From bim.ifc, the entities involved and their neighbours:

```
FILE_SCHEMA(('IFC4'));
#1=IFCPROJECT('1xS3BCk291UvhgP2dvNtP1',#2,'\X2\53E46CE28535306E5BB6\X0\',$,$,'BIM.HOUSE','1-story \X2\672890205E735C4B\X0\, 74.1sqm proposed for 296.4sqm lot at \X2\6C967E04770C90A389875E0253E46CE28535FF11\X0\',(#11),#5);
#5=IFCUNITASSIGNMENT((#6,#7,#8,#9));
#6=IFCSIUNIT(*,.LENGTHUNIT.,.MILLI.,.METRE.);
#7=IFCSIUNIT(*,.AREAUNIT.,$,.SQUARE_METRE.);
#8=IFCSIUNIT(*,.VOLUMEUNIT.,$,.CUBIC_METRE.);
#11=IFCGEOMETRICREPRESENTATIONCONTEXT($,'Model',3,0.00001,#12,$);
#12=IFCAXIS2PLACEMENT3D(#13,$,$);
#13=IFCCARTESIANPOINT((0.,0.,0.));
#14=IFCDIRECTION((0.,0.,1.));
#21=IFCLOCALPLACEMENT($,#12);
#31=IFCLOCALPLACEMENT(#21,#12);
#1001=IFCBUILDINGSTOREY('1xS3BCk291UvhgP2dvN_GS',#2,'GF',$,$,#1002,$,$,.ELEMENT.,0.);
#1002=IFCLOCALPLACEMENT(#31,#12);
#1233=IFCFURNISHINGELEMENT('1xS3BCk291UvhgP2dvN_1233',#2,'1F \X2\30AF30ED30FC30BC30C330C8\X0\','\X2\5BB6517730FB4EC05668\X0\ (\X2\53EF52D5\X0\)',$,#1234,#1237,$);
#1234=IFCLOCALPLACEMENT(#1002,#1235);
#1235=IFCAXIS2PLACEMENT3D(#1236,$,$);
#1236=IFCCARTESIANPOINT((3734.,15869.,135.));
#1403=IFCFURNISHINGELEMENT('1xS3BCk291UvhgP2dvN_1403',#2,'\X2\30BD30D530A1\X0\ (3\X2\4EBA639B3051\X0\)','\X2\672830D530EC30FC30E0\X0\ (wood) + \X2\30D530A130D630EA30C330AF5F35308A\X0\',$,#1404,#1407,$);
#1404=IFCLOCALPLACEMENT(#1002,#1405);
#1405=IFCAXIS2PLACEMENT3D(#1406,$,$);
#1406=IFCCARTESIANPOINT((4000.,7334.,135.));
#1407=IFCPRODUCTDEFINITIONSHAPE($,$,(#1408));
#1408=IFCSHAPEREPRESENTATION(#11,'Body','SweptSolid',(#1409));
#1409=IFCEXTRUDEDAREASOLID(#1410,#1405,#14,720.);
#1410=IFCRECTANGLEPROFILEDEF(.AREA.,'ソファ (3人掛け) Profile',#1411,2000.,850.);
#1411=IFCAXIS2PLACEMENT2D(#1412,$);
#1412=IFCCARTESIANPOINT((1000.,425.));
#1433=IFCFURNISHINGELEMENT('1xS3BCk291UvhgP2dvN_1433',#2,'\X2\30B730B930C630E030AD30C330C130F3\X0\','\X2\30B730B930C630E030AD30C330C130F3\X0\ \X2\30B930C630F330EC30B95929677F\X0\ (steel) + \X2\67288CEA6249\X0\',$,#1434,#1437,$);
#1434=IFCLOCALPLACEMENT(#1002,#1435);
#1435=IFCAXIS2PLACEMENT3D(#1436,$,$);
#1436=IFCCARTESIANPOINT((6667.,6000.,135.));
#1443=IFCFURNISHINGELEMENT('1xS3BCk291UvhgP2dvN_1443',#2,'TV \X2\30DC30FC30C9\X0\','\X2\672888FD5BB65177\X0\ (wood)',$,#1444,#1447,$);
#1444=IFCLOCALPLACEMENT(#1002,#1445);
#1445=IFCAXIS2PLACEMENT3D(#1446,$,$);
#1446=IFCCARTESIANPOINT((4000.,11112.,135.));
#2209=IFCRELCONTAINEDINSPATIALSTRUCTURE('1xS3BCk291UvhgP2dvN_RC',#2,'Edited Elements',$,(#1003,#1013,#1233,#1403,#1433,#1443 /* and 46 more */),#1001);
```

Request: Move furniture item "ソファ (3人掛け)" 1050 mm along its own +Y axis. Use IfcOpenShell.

```python
import ifcopenshell
import ifcopenshell.api.geometry
import ifcopenshell.util.placement
import ifcopenshell.util.unit

model = ifcopenshell.open("bim.ifc")
unit_scale = ifcopenshell.util.unit.calculate_unit_scale(model)

item = model.by_id(1403)
matrix = ifcopenshell.util.placement.get_local_placement(item.ObjectPlacement)
matrix[:3, 3] += matrix[:3, 1] * 1.05 / unit_scale
ifcopenshell.api.geometry.edit_object_placement(model, product=item, matrix=matrix, is_si=False)

print(ifcopenshell.util.placement.get_local_placement(item.ObjectPlacement).round(3) + 0.0)

model.write("bim_v2.ifc")
```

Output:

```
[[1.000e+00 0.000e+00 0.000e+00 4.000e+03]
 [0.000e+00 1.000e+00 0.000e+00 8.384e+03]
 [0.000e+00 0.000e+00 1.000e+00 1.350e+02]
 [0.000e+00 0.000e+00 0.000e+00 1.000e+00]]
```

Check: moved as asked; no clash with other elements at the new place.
